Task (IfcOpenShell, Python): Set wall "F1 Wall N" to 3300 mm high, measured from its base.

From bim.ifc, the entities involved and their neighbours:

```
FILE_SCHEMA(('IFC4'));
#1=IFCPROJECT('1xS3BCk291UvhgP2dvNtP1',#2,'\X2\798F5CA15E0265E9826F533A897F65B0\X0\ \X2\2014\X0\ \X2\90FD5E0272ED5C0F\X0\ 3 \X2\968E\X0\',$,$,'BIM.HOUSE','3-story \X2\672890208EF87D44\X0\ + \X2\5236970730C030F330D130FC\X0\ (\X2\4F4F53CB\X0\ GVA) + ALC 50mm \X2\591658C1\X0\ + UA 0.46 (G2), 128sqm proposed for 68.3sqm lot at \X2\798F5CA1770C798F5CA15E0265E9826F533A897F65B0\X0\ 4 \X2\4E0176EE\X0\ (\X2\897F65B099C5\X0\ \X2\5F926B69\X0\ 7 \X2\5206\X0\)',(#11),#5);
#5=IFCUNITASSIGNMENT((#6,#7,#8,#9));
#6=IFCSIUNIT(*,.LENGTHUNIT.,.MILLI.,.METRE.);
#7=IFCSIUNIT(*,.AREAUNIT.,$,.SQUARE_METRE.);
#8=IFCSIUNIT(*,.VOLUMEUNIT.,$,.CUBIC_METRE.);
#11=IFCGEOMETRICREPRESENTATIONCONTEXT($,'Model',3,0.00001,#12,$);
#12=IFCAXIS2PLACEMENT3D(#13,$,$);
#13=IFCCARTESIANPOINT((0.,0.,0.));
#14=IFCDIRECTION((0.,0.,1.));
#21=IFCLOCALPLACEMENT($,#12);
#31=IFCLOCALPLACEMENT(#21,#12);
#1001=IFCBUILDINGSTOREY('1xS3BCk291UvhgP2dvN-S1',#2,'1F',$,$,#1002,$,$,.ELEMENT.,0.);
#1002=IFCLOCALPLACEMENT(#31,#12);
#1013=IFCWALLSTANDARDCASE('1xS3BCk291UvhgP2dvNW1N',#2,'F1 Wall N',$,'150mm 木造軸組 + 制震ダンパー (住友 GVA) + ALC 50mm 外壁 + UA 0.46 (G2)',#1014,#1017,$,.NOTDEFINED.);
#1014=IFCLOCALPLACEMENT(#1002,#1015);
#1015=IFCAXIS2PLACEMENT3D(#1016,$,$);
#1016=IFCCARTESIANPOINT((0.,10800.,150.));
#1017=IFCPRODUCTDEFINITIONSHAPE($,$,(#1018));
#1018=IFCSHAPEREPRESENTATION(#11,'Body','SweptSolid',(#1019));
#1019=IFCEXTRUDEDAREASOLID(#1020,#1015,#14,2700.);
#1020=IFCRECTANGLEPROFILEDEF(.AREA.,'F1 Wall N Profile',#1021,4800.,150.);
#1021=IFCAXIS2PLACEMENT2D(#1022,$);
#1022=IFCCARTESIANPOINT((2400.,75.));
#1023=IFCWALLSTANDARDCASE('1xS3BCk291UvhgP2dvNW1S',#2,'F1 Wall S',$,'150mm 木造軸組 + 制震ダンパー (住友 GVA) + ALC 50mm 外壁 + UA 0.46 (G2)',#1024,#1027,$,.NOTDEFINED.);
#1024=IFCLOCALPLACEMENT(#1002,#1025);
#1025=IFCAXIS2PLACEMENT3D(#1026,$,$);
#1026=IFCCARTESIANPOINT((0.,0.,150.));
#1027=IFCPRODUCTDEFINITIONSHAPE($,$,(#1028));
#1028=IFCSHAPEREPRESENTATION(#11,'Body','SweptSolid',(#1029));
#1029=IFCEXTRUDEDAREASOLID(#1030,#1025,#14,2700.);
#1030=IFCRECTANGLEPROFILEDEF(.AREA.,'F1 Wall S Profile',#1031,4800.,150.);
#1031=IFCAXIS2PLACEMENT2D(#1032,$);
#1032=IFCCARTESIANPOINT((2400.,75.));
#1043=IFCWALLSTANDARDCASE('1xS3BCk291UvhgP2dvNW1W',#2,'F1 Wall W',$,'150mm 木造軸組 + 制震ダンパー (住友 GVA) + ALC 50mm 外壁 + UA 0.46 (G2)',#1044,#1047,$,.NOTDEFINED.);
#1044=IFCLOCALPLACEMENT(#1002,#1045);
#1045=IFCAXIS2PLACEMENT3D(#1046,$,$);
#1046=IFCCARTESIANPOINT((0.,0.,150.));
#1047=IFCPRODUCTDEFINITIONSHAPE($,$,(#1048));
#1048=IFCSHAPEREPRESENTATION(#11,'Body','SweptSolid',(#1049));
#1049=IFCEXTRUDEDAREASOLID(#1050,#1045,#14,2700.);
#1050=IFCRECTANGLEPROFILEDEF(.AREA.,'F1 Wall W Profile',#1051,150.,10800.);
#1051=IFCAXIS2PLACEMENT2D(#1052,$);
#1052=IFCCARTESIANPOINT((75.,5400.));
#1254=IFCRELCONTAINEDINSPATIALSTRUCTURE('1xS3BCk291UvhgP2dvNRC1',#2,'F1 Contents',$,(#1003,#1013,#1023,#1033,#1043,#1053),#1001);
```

```python
import ifcopenshell
import ifcopenshell.geom
import ifcopenshell.util.shape
import ifcopenshell.util.unit

model = ifcopenshell.open("bim.ifc")
unit_scale = ifcopenshell.util.unit.calculate_unit_scale(model)
settings = ifcopenshell.geom.settings()


def volume(element):
    """Net volume in cubic metres, openings subtracted."""
    shape = ifcopenshell.geom.create_shape(settings, element)
    return ifcopenshell.util.shape.get_volume(shape.geometry)


wall = model.by_id(1013)
before = volume(wall)

body = next(r for r in wall.Representation.Representations if r.RepresentationIdentifier == "Body")
solid = body.Items[0]
old_height = solid.Depth
solid.Depth = 3.3 / unit_scale
after = volume(wall)

print(f"height {old_height:g} -> {solid.Depth:g}, volume {before:.3f} -> {after:.3f} m3")

model.write("bim-out.ifc")
```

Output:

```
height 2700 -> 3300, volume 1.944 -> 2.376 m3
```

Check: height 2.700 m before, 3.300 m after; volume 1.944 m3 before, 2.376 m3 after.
